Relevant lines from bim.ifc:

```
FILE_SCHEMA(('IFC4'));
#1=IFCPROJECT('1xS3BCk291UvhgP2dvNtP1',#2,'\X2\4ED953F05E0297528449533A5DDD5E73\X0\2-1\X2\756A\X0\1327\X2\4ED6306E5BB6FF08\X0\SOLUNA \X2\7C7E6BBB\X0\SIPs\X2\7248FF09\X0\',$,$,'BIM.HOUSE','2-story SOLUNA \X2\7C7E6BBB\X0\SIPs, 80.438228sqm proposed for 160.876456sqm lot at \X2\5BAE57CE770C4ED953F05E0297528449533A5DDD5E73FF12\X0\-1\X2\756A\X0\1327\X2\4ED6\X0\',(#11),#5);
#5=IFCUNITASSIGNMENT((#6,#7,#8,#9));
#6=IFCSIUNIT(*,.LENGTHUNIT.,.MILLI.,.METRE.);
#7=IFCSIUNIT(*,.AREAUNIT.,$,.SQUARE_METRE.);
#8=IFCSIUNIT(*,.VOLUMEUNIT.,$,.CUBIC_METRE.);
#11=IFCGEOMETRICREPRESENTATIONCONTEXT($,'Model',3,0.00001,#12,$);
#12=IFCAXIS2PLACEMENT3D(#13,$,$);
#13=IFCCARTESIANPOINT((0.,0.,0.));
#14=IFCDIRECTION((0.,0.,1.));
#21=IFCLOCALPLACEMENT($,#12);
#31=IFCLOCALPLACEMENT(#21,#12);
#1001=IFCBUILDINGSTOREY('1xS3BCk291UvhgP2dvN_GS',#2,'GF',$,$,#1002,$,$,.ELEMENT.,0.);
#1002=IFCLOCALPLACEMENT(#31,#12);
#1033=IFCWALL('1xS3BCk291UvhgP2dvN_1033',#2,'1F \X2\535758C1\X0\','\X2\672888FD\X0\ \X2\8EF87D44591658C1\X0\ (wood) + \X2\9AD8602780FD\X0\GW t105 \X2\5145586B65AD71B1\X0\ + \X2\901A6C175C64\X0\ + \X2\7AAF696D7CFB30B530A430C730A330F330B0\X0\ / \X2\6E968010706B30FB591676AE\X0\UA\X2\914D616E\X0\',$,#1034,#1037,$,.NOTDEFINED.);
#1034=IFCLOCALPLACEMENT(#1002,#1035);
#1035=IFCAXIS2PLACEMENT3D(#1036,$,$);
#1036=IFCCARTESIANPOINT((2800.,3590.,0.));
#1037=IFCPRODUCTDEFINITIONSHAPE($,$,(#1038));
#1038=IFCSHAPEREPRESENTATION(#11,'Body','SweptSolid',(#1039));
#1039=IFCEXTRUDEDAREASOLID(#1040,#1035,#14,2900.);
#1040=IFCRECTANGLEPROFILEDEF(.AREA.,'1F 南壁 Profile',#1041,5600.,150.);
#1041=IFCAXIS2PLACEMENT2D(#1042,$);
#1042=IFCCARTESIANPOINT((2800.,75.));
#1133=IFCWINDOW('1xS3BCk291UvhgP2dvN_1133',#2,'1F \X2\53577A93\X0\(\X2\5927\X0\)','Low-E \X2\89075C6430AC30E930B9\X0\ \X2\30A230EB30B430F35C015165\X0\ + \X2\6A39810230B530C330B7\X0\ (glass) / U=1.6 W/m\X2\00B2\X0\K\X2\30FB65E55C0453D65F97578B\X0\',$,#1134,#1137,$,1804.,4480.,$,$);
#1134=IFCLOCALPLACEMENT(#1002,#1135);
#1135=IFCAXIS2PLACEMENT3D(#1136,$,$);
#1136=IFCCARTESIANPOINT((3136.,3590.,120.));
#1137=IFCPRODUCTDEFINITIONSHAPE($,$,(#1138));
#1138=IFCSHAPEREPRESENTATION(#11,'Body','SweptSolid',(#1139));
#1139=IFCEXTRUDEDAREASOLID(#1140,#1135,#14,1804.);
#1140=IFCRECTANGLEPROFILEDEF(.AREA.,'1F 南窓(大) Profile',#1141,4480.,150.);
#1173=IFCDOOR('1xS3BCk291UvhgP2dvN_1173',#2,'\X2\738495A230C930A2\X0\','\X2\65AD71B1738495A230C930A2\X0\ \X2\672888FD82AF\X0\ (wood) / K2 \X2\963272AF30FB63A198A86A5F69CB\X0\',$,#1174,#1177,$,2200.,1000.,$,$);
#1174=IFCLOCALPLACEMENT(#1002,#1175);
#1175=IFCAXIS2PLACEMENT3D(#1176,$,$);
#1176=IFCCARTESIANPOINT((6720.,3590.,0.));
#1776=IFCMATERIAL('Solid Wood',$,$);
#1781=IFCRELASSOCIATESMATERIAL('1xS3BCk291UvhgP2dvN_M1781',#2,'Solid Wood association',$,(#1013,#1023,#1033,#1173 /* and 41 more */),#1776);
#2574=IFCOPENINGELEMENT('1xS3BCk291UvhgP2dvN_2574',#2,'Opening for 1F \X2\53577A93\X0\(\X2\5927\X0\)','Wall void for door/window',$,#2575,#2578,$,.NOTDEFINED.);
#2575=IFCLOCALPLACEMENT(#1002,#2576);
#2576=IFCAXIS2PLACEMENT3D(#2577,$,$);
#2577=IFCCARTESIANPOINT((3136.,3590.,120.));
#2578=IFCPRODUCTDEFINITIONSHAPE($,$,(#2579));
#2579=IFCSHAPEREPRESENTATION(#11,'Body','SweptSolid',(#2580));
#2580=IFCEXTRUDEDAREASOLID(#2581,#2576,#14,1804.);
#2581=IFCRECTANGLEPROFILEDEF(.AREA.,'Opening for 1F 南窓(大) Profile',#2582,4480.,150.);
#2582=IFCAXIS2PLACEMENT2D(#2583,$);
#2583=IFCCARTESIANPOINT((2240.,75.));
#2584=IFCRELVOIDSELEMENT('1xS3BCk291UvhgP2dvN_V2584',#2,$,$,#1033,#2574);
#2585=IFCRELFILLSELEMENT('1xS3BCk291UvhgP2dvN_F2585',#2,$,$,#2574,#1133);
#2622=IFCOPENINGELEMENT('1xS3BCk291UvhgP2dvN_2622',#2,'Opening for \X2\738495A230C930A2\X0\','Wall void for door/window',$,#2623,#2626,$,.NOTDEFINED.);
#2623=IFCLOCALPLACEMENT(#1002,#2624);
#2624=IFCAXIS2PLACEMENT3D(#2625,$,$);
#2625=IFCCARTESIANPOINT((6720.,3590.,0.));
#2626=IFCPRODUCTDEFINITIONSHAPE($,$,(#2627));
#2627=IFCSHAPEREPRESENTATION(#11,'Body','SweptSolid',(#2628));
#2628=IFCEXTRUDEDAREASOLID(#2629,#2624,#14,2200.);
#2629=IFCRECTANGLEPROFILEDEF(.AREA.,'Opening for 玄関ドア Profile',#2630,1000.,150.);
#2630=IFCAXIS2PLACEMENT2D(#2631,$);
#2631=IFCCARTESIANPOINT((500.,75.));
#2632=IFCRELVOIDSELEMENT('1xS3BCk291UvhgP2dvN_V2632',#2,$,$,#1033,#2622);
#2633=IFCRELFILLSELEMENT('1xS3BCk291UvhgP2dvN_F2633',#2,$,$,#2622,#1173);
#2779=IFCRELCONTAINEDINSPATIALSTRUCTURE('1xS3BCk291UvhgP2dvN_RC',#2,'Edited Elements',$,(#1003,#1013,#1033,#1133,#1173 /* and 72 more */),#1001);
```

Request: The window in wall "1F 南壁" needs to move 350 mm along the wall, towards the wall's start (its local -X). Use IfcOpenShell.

```python
import ifcopenshell
import ifcopenshell.api.geometry
import ifcopenshell.util.placement

model = ifcopenshell.open("bim.ifc")

window = model.by_id(1133)
opening = window.FillsVoids[0].RelatingOpeningElement
wall = opening.VoidsElements[0].RelatingBuildingElement

wall_matrix = ifcopenshell.util.placement.get_local_placement(wall.ObjectPlacement)
shift = wall_matrix[:3, 0] * -350.0
before = ifcopenshell.util.placement.get_local_placement(window.ObjectPlacement)[:3, 3].copy()

# The window is not placed relative to its opening, so move both.
for product in (opening, window):
    matrix = ifcopenshell.util.placement.get_local_placement(product.ObjectPlacement)
    matrix[:3, 3] += shift
    ifcopenshell.api.geometry.edit_object_placement(model, product=product, matrix=matrix, is_si=False)

after = ifcopenshell.util.placement.get_local_placement(window.ObjectPlacement)[:3, 3]
print("window moved by", (after - before).round(3) + 0.0)

model.write("bim_updated.ifc")
```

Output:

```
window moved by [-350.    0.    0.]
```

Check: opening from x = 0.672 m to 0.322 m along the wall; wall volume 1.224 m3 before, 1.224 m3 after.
